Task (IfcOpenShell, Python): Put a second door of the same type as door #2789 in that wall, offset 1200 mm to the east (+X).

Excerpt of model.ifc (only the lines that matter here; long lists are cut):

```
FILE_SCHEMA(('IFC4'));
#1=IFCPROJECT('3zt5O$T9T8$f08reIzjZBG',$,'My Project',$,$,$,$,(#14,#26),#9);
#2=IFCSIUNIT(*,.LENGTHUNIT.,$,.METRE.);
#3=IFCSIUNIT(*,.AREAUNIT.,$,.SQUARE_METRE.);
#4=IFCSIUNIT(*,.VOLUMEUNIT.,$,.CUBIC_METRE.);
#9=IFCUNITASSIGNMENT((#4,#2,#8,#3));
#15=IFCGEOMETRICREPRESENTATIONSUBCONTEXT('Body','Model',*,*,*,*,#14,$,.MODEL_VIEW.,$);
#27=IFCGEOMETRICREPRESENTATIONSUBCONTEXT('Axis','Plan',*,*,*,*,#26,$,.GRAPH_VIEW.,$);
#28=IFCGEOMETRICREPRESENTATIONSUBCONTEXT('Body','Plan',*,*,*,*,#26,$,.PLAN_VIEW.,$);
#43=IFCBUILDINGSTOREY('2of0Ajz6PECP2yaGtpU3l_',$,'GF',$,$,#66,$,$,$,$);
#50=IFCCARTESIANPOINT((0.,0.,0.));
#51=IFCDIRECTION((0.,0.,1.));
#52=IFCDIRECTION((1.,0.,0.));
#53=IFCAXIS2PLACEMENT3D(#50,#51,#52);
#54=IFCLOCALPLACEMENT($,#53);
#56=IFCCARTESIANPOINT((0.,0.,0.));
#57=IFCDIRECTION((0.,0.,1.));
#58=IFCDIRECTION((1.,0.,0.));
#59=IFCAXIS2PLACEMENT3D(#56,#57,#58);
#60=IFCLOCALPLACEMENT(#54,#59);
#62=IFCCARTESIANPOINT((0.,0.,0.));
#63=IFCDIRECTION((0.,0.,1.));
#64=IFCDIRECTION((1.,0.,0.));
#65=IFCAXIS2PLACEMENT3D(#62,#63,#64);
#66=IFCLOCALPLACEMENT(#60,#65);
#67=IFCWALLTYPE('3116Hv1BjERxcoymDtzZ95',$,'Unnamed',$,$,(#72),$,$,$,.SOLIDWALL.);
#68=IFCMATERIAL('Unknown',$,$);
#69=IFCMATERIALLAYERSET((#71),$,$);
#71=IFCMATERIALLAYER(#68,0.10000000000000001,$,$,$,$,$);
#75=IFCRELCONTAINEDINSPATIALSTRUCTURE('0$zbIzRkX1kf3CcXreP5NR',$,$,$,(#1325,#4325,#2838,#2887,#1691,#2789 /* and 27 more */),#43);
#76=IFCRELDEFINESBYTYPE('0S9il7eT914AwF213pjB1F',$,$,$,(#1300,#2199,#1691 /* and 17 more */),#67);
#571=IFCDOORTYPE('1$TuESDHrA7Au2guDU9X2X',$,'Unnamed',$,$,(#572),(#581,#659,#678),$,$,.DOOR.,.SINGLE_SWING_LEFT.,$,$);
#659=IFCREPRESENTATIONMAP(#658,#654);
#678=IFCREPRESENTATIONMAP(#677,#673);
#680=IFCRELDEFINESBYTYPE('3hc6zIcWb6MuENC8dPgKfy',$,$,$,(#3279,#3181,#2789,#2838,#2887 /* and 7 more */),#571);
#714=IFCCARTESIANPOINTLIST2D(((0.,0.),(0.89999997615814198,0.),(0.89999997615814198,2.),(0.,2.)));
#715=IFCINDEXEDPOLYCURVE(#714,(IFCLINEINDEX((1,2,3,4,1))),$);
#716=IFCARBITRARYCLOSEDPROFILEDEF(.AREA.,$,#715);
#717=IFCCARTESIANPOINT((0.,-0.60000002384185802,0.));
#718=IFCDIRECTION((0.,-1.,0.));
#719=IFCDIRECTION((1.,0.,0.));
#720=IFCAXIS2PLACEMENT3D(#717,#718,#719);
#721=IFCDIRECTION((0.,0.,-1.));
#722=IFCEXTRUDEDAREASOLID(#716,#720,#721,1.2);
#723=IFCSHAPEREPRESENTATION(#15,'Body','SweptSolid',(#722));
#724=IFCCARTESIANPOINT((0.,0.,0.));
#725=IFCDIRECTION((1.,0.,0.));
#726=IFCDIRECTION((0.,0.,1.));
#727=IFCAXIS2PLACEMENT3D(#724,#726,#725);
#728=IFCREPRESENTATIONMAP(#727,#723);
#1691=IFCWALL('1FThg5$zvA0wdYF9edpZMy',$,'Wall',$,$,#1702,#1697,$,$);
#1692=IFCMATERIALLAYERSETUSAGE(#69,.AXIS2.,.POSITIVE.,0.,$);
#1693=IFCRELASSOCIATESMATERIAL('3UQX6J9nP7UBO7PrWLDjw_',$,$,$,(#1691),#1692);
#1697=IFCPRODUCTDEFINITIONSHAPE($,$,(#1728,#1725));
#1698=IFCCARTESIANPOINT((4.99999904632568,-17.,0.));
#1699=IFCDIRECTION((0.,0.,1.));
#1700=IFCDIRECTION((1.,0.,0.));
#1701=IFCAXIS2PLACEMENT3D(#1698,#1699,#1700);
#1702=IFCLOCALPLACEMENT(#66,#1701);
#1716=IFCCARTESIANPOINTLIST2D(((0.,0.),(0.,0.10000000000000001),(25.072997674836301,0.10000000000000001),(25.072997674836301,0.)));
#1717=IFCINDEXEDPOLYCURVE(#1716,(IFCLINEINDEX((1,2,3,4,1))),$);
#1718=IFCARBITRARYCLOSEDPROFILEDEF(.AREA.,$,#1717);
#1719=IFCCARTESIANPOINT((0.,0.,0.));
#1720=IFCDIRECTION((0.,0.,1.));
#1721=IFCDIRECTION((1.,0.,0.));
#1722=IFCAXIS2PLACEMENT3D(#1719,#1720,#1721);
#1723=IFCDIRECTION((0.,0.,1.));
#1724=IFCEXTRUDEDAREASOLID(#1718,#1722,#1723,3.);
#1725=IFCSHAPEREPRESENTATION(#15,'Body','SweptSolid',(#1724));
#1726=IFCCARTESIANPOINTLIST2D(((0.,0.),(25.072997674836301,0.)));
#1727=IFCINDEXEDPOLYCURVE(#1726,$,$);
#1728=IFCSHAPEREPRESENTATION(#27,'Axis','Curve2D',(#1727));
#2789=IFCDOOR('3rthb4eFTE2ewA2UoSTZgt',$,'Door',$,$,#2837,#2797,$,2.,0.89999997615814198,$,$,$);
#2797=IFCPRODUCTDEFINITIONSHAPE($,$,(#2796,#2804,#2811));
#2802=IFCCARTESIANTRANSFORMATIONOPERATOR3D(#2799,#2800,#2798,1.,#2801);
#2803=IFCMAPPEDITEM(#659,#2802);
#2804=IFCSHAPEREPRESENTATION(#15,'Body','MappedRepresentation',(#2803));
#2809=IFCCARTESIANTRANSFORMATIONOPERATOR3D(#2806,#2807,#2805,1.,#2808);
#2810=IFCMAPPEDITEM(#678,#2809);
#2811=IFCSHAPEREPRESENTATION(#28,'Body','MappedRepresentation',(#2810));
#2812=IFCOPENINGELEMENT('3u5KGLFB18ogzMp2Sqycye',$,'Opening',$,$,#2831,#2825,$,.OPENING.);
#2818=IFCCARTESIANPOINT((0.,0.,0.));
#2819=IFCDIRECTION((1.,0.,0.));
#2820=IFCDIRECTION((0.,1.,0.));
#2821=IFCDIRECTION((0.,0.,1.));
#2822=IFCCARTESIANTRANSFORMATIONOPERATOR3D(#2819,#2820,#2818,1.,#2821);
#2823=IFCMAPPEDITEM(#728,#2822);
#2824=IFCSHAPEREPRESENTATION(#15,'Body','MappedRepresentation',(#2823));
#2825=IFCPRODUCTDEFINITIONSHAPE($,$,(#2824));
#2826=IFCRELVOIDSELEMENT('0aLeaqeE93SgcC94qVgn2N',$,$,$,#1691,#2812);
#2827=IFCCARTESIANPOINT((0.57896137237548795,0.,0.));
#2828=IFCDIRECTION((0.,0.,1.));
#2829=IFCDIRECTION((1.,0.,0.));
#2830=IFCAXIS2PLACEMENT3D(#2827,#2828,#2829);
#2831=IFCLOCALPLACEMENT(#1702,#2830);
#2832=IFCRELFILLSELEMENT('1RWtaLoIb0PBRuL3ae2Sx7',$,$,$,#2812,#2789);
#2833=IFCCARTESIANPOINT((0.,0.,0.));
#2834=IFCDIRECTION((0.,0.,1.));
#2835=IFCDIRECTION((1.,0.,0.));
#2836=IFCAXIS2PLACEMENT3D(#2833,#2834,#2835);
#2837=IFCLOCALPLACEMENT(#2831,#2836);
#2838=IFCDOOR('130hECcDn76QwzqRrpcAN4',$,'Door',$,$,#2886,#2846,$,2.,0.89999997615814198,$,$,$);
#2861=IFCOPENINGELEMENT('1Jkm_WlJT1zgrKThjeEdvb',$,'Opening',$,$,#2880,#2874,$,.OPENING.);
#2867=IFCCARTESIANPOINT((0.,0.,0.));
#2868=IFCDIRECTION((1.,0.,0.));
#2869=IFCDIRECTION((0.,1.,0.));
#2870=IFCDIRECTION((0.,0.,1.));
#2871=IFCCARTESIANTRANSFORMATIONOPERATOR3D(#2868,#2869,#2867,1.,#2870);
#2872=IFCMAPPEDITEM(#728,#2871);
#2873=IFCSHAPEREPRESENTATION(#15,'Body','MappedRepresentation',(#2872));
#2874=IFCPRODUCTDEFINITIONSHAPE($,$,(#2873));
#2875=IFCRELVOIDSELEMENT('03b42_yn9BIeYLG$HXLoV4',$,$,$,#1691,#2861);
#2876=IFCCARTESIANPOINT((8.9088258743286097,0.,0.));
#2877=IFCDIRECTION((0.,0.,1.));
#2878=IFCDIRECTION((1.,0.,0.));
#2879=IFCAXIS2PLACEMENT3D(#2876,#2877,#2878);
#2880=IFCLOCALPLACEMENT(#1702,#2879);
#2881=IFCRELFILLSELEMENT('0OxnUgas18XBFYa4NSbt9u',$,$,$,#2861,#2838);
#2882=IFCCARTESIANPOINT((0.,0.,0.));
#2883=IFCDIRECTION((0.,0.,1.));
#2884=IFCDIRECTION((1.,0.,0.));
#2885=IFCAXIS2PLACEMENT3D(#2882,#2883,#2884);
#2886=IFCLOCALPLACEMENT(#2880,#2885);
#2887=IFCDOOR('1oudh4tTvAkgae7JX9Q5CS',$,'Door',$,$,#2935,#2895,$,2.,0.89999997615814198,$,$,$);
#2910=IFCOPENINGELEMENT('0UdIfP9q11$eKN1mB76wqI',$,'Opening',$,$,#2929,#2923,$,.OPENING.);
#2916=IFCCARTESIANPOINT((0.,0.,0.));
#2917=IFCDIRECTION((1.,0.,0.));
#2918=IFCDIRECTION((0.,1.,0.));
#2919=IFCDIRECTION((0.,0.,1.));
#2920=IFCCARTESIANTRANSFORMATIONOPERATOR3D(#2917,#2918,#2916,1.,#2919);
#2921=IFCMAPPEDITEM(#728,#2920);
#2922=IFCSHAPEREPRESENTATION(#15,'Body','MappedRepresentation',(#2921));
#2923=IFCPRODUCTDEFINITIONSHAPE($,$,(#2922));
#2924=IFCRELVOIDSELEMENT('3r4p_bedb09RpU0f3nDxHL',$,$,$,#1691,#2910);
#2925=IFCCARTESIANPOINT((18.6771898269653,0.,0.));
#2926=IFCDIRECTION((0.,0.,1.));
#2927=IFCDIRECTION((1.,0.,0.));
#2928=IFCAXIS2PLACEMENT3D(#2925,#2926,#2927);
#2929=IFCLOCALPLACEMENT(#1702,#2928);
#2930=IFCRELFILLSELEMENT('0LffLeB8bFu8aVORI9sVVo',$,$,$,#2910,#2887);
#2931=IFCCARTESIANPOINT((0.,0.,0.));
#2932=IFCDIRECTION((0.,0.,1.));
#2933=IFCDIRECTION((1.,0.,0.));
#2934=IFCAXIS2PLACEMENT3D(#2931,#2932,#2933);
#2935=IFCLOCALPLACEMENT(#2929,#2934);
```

```python
import ifcopenshell
import ifcopenshell.api.feature
import ifcopenshell.api.geometry
import ifcopenshell.api.root
import ifcopenshell.geom
import ifcopenshell.util.element
import ifcopenshell.util.placement
import ifcopenshell.util.shape

model = ifcopenshell.open("model.ifc")
settings = ifcopenshell.geom.settings()


def volume(element):
    """Net volume in cubic metres, openings subtracted."""
    shape = ifcopenshell.geom.create_shape(settings, element)
    return ifcopenshell.util.shape.get_volume(shape.geometry)


door = model.by_guid("3rthb4eFTE2ewA2UoSTZgt")
opening = door.FillsVoids[0].RelatingOpeningElement
wall = opening.VoidsElements[0].RelatingBuildingElement
before = volume(wall)
shift = ifcopenshell.util.placement.get_local_placement(wall.ObjectPlacement)[:3, 0] * 1.2

# copy_class copies the void relationship, type, container and properties, but no geometry.
new_opening = ifcopenshell.api.root.copy_class(model, product=opening)
new_opening.Representation = ifcopenshell.util.element.copy_deep(
    model, opening.Representation, exclude=["IfcGeometricRepresentationContext", "IfcRepresentationMap"]
)
new_door = ifcopenshell.api.root.copy_class(model, product=door)
new_door.Representation = ifcopenshell.util.element.copy_deep(
    model, door.Representation, exclude=["IfcGeometricRepresentationContext", "IfcRepresentationMap"]
)
ifcopenshell.api.feature.add_filling(model, opening=new_opening, element=new_door)

for old, new in ((opening, new_opening), (door, new_door)):
    matrix = ifcopenshell.util.placement.get_local_placement(old.ObjectPlacement)
    matrix[:3, 3] += shift
    ifcopenshell.api.geometry.edit_object_placement(model, product=new, matrix=matrix, is_si=False)

after = volume(wall)

print(f"wall volume {before:.3f} -> {after:.3f} m3")

model.write("model_edited.ifc")
```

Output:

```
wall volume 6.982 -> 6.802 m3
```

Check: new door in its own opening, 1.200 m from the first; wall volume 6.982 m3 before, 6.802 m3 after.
